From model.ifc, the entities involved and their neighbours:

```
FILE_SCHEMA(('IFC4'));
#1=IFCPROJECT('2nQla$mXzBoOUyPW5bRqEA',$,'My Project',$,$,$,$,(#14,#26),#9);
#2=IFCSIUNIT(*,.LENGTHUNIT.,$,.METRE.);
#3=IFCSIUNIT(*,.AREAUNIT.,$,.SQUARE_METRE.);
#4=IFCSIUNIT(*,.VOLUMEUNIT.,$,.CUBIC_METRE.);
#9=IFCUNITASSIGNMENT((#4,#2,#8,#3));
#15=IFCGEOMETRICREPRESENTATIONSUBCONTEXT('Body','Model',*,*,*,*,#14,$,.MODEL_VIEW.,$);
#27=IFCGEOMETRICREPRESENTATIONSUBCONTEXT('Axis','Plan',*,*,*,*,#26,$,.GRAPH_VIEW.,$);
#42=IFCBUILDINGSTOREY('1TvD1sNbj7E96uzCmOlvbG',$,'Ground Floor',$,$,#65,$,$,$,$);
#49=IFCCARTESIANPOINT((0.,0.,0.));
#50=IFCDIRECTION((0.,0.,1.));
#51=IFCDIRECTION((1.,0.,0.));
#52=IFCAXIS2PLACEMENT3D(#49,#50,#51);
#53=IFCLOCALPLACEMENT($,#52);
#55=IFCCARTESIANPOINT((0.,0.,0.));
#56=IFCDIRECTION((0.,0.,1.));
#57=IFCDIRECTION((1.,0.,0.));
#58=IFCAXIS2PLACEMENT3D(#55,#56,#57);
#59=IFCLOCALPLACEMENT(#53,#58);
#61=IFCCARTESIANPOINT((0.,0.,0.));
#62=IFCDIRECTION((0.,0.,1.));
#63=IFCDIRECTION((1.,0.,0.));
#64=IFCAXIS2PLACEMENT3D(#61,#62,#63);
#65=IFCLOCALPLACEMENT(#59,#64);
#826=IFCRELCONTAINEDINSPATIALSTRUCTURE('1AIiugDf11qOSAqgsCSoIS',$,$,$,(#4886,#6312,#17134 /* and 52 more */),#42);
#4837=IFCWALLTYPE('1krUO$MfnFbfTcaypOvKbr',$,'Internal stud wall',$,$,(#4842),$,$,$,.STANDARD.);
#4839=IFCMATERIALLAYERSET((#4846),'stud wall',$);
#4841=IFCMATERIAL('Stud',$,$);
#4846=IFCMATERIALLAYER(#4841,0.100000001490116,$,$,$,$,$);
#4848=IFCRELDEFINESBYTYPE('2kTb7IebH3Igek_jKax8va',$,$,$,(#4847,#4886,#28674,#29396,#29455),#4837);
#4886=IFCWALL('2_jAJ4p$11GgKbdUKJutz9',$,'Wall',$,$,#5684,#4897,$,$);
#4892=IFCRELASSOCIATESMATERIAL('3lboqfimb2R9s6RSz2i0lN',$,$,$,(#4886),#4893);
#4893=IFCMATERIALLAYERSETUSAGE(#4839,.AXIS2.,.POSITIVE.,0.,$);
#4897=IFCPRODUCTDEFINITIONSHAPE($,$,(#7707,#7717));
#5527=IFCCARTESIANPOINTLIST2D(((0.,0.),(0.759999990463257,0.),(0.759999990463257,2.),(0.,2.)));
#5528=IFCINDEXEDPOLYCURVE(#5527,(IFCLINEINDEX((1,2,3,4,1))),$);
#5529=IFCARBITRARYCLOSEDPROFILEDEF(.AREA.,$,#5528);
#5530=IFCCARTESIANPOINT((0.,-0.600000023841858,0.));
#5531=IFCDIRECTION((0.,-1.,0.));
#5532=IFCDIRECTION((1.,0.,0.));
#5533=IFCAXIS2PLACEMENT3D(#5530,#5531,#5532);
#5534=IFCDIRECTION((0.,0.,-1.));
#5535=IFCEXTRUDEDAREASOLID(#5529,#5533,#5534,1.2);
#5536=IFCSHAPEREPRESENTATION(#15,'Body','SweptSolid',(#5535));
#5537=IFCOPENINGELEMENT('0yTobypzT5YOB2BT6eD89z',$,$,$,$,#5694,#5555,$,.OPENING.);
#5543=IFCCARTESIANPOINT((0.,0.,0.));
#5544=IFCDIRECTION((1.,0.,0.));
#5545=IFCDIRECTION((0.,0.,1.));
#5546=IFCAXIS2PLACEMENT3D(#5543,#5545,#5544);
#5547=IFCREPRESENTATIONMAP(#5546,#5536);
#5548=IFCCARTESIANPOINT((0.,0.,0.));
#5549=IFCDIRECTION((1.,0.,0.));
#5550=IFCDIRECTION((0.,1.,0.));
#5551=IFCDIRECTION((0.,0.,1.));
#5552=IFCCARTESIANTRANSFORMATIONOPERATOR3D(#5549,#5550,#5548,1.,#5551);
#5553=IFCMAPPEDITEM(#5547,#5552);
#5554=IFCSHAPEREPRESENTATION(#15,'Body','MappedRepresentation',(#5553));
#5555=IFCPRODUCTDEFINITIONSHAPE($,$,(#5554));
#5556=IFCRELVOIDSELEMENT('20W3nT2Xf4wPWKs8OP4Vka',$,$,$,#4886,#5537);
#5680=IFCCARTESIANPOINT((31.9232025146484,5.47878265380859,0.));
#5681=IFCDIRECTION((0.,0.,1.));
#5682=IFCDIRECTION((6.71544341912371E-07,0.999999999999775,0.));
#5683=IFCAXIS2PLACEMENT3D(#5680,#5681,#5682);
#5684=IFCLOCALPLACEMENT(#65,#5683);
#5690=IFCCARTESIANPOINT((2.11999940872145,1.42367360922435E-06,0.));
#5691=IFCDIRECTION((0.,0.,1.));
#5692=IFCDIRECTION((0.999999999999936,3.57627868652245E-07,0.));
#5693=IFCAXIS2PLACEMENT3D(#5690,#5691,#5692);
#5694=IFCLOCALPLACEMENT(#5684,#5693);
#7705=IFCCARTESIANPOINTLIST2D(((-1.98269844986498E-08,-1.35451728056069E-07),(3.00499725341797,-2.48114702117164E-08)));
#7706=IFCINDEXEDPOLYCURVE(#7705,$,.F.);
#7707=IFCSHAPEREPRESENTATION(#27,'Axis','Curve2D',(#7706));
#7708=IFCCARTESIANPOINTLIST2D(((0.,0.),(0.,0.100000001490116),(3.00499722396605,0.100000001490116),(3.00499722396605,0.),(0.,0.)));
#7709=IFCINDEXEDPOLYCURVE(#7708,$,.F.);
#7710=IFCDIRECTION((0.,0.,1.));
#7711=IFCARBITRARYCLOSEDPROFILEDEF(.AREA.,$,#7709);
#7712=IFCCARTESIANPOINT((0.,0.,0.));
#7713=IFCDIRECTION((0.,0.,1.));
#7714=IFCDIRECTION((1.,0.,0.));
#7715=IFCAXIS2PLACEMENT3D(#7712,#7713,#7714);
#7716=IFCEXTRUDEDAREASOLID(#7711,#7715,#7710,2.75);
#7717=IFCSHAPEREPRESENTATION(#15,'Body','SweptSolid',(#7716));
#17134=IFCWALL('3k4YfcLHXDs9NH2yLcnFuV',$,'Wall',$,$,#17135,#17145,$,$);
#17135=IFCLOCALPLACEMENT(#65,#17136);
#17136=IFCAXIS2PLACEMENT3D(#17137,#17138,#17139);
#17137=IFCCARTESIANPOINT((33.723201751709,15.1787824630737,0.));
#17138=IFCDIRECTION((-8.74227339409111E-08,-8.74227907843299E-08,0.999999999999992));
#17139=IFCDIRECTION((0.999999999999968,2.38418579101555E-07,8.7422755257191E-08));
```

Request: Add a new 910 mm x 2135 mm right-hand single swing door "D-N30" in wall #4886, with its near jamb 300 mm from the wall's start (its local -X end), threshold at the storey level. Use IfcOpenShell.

```python
import numpy as np
import ifcopenshell
import ifcopenshell.api.feature
import ifcopenshell.api.geometry
import ifcopenshell.api.root
import ifcopenshell.api.spatial
import ifcopenshell.geom
import ifcopenshell.util.element
import ifcopenshell.util.placement
import ifcopenshell.util.representation
import ifcopenshell.util.shape
import ifcopenshell.util.unit

model = ifcopenshell.open("model.ifc")
unit_scale = ifcopenshell.util.unit.calculate_unit_scale(model)
settings = ifcopenshell.geom.settings()


def volume(element):
    """Net volume in cubic metres, openings subtracted."""
    shape = ifcopenshell.geom.create_shape(settings, element)
    return ifcopenshell.util.shape.get_volume(shape.geometry)


wall = model.by_id(4886)
storey = ifcopenshell.util.element.get_container(wall, ifc_class="IfcBuildingStorey")
context = ifcopenshell.util.representation.get_context(model, "Model", "Body", "MODEL_VIEW")
before = volume(wall)

width, height, from_end, sill = 0.91, 2.135, 0.3, 0.0  # metres

# The wall runs along its own X axis, and the end named is its -X end.
wall_shape = ifcopenshell.geom.create_shape(settings, wall)
x, y, z = ifcopenshell.util.shape.get_vertices(wall_shape.geometry).T
start = x.min() + from_end
face, thickness = float(y.min()), float(y.max() - y.min())
wall_matrix = ifcopenshell.util.placement.get_local_placement(wall.ObjectPlacement)
level = ifcopenshell.util.placement.get_local_placement(storey.ObjectPlacement)[2, 3]


def in_wall(x, y):
    """Placement at x, y metres in the wall's axes, at sill height."""
    matrix = wall_matrix.copy()
    matrix[:, 3] = wall_matrix @ np.array([x / unit_scale, y / unit_scale, 0.0, 1.0])
    matrix[2, 3] = level + sill / unit_scale
    return matrix


# Opening: a box that overshoots both wall faces by 50 mm.
opening = ifcopenshell.api.root.create_entity(model, ifc_class="IfcOpeningElement", predefined_type="OPENING")
box = ifcopenshell.api.geometry.add_wall_representation(
    model, context=context, length=width, height=height, thickness=thickness + 0.1
)
ifcopenshell.api.geometry.assign_representation(model, product=opening, representation=box)
ifcopenshell.api.geometry.edit_object_placement(model, product=opening, matrix=in_wall(start, face - 0.05), is_si=False)
ifcopenshell.api.feature.add_feature(model, feature=opening, element=wall)

door = ifcopenshell.api.root.create_entity(model, ifc_class="IfcDoor", name="D-N30", predefined_type="DOOR")
door.OverallWidth, door.OverallHeight = width / unit_scale, height / unit_scale
door.OperationType = "SINGLE_SWING_RIGHT"
body = ifcopenshell.api.geometry.add_door_representation(
    model,
    context=context,
    overall_width=door.OverallWidth,
    overall_height=door.OverallHeight,
    operation_type="SINGLE_SWING_RIGHT",
    lining_properties={"LiningDepth": thickness / unit_scale, "ThresholdDepth": thickness / unit_scale},
)
ifcopenshell.api.geometry.assign_representation(model, product=door, representation=body)
ifcopenshell.api.spatial.assign_container(model, products=[door], relating_structure=storey)
ifcopenshell.api.feature.add_filling(model, opening=opening, element=door)

# The lining spans the wall, so the door starts at the wall face.
ifcopenshell.api.geometry.edit_object_placement(model, product=door, matrix=in_wall(start, face), is_si=False)

after = volume(wall)

print(f"wall volume {before:.3f} -> {after:.3f} m3")

model.write("model_updated.ifc")
```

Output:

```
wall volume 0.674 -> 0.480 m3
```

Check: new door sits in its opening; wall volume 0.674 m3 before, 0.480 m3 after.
